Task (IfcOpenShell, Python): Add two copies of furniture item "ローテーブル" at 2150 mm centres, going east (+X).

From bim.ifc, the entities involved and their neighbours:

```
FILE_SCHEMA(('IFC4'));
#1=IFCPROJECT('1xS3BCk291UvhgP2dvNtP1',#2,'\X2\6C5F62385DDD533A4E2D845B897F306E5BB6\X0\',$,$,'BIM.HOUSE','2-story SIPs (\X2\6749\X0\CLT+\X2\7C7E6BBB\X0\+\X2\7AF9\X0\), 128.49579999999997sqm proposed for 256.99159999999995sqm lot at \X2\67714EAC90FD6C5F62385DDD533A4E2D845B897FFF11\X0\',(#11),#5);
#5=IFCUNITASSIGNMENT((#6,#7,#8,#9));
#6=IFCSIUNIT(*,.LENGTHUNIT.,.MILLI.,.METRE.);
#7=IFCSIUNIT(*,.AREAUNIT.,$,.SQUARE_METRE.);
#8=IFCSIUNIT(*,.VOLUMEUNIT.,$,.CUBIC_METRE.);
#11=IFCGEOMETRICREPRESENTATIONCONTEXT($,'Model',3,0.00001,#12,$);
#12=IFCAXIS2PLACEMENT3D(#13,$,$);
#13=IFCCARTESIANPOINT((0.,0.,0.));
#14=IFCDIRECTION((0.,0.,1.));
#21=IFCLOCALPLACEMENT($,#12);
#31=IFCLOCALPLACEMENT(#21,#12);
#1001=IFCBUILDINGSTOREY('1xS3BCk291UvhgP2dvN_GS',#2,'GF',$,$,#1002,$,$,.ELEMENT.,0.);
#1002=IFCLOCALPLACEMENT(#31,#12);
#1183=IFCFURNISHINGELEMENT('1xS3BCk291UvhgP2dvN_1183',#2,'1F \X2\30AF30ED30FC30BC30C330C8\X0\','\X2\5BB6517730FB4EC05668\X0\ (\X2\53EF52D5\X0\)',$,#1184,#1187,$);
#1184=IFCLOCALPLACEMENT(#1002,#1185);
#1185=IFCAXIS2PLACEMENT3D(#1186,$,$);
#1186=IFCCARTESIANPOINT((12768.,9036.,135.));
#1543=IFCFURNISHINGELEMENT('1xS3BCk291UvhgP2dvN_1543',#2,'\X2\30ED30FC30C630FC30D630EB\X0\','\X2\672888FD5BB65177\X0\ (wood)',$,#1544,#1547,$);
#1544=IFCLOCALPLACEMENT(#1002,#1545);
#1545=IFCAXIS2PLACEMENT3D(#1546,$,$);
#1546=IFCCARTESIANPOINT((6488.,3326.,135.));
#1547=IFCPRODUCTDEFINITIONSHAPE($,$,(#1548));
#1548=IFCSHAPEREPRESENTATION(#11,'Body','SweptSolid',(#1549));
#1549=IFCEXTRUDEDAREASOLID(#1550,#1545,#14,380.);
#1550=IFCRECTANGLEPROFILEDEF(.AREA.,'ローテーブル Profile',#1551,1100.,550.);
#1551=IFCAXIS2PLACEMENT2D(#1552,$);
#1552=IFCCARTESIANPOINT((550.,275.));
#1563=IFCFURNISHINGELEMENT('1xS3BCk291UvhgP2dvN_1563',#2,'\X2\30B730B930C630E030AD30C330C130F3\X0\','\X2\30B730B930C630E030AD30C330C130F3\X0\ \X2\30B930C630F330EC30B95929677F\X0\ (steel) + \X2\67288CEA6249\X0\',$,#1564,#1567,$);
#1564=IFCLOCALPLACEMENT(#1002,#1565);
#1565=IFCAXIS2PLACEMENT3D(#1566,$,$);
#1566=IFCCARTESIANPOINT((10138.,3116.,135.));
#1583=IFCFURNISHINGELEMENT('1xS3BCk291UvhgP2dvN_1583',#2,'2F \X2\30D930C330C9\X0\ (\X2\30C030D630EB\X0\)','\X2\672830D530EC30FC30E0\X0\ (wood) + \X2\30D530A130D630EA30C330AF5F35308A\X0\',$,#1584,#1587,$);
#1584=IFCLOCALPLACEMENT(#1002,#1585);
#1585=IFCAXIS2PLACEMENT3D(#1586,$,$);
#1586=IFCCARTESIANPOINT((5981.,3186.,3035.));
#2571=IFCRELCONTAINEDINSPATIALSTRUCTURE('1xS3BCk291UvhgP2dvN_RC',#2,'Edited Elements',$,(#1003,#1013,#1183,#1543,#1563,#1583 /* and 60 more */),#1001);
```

```python
import numpy as np
import ifcopenshell
import ifcopenshell.api.geometry
import ifcopenshell.api.root
import ifcopenshell.util.element
import ifcopenshell.util.placement
import ifcopenshell.util.unit

model = ifcopenshell.open("bim.ifc")
unit_scale = ifcopenshell.util.unit.calculate_unit_scale(model)


def reuse_history(source, copy):
    """copy_class also copies each property set's owner history, people and application; keep the originals."""
    for rel in copy.IsDefinedBy:
        if rel.is_a("IfcRelDefinesByProperties") and (history := rel.RelatingPropertyDefinition.OwnerHistory):
            rel.RelatingPropertyDefinition.OwnerHistory = source.OwnerHistory
            ifcopenshell.util.element.remove_deep2(model, history)


source = model.by_id(1543)
base = ifcopenshell.util.placement.get_local_placement(source.ObjectPlacement)
step = np.array([1.0, 0.0, 0.0]) * 2.15 / unit_scale

for i in range(1, 3):
    copy = ifcopenshell.api.root.copy_class(model, product=source)
    copy.Representation = ifcopenshell.util.element.copy_deep(
        model, source.Representation, exclude=["IfcGeometricRepresentationContext", "IfcRepresentationMap"]
    )
    reuse_history(source, copy)
    matrix = base.copy()
    matrix[:3, 3] += i * step
    print("added at", matrix[:3, 3].round(3) + 0.0)
    ifcopenshell.api.geometry.edit_object_placement(model, product=copy, matrix=matrix, is_si=False)

model.write("bim_rev.ifc")
```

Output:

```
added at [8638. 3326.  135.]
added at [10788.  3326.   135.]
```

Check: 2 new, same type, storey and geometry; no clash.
